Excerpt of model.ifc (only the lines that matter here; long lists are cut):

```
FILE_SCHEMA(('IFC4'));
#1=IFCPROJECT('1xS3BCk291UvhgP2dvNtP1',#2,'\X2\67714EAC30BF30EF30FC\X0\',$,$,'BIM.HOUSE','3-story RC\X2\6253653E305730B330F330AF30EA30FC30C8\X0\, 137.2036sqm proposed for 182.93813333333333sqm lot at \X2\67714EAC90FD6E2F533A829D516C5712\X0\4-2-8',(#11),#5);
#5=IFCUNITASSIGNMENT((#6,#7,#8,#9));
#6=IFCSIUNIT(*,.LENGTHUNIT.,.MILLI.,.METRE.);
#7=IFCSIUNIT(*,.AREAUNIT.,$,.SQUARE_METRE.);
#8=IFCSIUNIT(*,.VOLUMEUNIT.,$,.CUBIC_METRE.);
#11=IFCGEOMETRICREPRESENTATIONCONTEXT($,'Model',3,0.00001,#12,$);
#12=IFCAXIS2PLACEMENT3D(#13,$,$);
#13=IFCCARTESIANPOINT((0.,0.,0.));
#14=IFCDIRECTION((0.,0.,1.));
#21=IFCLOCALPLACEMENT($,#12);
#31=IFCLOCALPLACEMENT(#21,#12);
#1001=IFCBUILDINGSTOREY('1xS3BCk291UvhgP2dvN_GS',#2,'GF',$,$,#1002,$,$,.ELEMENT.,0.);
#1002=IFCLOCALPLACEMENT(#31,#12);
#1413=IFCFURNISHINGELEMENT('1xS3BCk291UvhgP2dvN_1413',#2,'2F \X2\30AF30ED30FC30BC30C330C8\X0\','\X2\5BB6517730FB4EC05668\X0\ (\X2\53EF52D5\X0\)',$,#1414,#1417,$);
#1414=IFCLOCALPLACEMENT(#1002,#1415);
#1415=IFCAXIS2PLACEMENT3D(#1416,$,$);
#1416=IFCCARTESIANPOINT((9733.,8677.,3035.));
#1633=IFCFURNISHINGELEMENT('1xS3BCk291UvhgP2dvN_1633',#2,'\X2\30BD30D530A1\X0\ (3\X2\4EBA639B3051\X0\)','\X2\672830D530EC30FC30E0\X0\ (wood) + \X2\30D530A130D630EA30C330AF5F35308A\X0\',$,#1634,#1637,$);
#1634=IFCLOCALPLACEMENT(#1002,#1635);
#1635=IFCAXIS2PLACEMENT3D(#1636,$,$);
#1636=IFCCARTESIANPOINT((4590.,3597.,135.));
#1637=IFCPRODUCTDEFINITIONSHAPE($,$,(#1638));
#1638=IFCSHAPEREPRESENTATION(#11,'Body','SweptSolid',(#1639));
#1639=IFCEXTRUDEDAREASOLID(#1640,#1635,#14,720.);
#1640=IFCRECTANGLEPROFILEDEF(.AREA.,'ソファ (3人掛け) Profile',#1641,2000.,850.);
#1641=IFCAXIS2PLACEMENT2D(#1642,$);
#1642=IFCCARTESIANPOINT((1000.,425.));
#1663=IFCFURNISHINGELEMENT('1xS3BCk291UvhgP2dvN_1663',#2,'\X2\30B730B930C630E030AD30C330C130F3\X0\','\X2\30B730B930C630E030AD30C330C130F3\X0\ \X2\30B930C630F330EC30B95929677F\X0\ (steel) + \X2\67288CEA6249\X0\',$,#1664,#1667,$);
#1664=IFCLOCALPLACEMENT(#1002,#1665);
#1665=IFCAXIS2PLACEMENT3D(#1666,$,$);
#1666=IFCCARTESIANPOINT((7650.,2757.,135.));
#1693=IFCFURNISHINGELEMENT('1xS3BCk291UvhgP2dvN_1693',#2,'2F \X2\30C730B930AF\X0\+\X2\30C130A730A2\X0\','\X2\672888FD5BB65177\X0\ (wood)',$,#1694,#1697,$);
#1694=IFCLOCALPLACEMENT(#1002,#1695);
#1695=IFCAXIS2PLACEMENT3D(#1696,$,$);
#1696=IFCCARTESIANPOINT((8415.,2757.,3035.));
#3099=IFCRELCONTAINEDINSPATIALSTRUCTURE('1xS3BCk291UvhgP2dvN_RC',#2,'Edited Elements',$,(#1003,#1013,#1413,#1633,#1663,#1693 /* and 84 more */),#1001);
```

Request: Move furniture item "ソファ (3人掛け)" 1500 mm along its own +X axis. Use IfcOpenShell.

```python
import ifcopenshell
import ifcopenshell.api.geometry
import ifcopenshell.util.placement

model = ifcopenshell.open("model.ifc")

item = model.by_id(1633)
matrix = ifcopenshell.util.placement.get_local_placement(item.ObjectPlacement)
matrix[:3, 3] += matrix[:3, 0] * 1500.0
ifcopenshell.api.geometry.edit_object_placement(model, product=item, matrix=matrix, is_si=False)

print(ifcopenshell.util.placement.get_local_placement(item.ObjectPlacement).round(3) + 0.0)

model.write("model_rev.ifc")
```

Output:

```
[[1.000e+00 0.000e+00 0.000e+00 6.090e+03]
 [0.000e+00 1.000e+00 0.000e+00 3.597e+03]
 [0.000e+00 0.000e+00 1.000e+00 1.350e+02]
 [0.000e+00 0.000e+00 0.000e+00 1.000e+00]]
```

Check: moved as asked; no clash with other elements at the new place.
